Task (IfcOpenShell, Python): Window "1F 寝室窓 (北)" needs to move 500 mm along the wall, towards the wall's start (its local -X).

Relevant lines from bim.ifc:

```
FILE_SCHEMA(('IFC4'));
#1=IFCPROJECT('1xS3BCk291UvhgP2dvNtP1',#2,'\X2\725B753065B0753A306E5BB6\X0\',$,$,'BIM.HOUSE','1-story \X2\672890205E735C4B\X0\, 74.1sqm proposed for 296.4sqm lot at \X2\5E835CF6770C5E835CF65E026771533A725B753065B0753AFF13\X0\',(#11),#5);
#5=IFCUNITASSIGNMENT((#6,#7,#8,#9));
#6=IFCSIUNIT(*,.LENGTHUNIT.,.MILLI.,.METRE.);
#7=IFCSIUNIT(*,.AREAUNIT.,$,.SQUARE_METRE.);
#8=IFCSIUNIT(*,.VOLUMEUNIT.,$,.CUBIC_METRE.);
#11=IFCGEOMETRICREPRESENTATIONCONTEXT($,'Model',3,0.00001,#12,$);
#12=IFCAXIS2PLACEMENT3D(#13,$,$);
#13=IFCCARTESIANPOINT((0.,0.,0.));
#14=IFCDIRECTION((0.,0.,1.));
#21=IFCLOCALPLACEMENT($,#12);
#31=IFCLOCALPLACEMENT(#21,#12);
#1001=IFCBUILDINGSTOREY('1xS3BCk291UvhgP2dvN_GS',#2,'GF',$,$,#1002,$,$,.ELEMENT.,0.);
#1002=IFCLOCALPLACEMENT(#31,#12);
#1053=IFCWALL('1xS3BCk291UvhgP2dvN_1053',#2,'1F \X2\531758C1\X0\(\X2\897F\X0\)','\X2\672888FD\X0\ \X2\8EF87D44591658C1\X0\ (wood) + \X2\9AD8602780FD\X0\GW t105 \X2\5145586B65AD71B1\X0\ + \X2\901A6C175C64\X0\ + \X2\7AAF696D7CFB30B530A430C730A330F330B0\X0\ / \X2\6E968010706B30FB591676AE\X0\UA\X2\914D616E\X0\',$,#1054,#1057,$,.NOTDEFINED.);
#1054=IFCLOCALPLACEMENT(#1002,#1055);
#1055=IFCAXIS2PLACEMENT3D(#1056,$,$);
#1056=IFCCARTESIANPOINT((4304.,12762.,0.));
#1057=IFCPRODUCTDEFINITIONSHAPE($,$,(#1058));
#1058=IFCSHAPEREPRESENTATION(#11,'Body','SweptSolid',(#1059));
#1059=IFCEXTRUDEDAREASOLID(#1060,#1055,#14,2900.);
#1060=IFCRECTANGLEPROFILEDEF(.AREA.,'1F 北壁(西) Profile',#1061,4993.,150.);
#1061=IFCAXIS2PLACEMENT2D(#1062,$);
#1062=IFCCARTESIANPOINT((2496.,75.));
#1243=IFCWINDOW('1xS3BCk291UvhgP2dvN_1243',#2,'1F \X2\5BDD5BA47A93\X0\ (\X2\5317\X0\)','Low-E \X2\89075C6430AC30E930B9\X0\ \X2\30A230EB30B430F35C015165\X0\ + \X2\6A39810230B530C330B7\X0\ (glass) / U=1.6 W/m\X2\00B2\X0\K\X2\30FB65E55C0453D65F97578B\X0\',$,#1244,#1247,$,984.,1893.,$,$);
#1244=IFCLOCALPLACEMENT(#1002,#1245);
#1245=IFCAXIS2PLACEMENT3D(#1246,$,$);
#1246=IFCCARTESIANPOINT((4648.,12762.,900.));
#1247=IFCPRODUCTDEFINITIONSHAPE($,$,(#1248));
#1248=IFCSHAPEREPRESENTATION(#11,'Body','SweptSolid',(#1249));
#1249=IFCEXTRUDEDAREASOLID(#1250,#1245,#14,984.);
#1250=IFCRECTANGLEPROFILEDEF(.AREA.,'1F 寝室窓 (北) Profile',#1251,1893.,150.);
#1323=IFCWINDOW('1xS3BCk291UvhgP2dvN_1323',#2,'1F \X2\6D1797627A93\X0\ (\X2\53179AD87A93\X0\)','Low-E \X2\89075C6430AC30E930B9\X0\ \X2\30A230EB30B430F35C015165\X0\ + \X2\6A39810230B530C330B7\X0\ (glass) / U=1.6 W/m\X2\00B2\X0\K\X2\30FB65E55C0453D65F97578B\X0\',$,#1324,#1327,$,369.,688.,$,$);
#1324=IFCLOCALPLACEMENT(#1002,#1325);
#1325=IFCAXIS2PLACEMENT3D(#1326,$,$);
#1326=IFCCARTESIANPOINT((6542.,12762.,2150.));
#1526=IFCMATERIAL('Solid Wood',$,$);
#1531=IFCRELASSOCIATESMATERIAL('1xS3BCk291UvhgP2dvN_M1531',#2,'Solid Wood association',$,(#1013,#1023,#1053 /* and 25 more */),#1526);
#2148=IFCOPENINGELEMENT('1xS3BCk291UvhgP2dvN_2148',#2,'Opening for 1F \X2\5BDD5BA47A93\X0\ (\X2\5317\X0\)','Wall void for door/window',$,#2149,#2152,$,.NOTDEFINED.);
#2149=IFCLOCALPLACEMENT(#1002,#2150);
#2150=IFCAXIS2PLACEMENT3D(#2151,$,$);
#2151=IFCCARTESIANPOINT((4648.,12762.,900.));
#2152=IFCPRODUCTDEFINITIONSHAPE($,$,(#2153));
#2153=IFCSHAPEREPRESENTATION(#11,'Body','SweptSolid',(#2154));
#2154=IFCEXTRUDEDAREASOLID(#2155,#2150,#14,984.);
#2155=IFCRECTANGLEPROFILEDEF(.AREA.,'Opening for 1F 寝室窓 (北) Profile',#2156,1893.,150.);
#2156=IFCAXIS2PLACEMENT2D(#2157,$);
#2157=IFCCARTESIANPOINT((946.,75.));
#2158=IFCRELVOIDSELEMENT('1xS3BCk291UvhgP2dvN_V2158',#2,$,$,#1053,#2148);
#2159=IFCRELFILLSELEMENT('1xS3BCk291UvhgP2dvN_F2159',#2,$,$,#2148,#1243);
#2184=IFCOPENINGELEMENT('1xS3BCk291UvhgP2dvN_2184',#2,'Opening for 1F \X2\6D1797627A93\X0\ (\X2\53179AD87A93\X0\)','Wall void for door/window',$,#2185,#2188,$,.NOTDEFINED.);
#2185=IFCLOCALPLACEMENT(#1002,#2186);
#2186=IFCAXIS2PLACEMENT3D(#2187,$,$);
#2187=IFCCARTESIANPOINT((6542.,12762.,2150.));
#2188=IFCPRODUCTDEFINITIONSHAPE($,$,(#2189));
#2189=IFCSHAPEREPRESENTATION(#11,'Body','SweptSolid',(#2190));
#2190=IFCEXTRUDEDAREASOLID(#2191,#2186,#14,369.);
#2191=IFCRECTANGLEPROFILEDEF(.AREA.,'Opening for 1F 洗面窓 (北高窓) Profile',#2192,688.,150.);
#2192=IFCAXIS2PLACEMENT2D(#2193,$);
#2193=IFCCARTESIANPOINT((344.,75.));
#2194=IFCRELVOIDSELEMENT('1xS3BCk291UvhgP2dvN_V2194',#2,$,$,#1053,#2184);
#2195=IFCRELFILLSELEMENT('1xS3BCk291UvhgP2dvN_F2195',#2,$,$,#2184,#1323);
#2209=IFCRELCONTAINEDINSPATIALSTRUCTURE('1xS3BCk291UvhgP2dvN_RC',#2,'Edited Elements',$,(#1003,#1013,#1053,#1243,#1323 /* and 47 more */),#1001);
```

```python
import ifcopenshell
import ifcopenshell.api.geometry
import ifcopenshell.util.placement
import ifcopenshell.util.unit

model = ifcopenshell.open("bim.ifc")
unit_scale = ifcopenshell.util.unit.calculate_unit_scale(model)

window = model.by_guid("1xS3BCk291UvhgP2dvN_1243")
opening = window.FillsVoids[0].RelatingOpeningElement
wall = opening.VoidsElements[0].RelatingBuildingElement

wall_matrix = ifcopenshell.util.placement.get_local_placement(wall.ObjectPlacement)
shift = wall_matrix[:3, 0] * -0.5 / unit_scale
before = ifcopenshell.util.placement.get_local_placement(window.ObjectPlacement)[:3, 3].copy()

# The window is not placed relative to its opening, so move both.
for product in (opening, window):
    matrix = ifcopenshell.util.placement.get_local_placement(product.ObjectPlacement)
    matrix[:3, 3] += shift
    ifcopenshell.api.geometry.edit_object_placement(model, product=product, matrix=matrix, is_si=False)

after = ifcopenshell.util.placement.get_local_placement(window.ObjectPlacement)[:3, 3]
print("window moved by", (after - before).round(3) + 0.0)

model.write("bim-out.ifc")
```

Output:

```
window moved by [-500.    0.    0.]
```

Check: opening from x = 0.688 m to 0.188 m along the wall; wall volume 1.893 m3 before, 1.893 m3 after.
